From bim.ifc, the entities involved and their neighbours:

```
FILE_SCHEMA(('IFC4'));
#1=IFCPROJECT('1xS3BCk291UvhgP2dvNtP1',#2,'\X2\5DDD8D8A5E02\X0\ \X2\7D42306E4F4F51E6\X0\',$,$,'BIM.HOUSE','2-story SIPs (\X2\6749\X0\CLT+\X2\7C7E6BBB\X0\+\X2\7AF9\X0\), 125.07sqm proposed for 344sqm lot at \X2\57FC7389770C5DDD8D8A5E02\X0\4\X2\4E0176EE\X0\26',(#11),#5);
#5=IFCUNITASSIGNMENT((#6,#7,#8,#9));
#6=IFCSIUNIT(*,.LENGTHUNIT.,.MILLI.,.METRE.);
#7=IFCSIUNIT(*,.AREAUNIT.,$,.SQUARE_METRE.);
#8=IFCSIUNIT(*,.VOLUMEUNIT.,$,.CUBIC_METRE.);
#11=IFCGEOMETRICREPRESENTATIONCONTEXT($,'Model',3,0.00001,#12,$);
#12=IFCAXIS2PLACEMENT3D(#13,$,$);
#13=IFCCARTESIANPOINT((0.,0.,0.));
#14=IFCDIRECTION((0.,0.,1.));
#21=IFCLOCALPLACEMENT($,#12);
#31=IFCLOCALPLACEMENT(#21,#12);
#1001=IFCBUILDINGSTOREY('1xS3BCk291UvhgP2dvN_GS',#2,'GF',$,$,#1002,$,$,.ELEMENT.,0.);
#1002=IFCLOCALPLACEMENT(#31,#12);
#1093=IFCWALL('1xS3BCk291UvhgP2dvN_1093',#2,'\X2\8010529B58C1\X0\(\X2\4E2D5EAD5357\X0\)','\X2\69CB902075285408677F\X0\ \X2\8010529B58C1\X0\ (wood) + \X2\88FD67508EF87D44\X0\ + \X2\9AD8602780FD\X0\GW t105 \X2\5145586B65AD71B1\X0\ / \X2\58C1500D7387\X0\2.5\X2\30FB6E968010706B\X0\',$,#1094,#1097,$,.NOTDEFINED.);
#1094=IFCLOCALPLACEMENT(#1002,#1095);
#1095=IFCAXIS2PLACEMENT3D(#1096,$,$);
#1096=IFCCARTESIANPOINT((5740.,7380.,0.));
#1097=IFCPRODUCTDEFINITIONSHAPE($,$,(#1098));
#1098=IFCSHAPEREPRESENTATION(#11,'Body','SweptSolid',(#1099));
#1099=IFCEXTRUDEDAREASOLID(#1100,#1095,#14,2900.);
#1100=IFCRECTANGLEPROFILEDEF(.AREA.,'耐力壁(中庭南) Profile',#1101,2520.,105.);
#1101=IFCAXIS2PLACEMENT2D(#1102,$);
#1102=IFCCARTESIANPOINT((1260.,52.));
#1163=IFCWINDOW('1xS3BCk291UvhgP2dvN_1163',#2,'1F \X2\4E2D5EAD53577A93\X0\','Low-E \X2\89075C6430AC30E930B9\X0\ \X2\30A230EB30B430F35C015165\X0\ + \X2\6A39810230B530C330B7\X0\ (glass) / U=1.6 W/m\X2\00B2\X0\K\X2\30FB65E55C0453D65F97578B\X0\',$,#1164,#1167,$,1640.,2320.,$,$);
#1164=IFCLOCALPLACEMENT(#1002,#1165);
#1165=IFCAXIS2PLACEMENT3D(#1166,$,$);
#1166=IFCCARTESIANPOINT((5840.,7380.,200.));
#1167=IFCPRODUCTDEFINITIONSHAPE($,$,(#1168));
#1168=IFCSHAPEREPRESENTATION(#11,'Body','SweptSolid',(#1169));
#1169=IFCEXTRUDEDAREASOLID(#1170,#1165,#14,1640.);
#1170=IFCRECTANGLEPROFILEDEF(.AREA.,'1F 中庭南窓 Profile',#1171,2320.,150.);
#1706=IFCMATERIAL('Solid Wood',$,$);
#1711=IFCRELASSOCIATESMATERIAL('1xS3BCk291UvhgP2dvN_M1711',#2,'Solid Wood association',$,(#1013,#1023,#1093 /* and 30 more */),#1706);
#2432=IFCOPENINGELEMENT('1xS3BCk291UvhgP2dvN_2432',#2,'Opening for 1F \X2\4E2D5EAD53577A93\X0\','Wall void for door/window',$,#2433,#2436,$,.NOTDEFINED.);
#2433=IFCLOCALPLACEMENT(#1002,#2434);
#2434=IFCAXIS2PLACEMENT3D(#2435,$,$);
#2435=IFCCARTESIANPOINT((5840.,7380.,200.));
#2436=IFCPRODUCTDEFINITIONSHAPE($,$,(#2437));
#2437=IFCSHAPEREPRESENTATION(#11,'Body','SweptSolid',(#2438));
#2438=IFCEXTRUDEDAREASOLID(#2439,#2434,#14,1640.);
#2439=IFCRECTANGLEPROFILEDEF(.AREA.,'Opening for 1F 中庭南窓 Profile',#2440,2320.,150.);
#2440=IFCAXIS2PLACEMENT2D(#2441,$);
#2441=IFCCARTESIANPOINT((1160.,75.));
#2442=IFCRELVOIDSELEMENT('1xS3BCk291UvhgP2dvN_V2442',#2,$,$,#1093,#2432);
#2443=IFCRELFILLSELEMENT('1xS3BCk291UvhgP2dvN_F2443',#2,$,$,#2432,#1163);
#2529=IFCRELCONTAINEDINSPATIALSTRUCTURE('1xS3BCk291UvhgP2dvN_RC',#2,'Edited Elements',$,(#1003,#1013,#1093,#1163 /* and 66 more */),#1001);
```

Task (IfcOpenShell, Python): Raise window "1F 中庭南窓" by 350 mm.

```python
import numpy as np
import ifcopenshell
import ifcopenshell.api.geometry
import ifcopenshell.util.placement
import ifcopenshell.util.unit

model = ifcopenshell.open("bim.ifc")
unit_scale = ifcopenshell.util.unit.calculate_unit_scale(model)

window = model.by_guid("1xS3BCk291UvhgP2dvN_1163")
opening = window.FillsVoids[0].RelatingOpeningElement
dz = 0.35 / unit_scale

shift = np.array([0.0, 0.0, dz])
# The window is not placed relative to its opening, so move both.
for product in (opening, window):
    matrix = ifcopenshell.util.placement.get_local_placement(product.ObjectPlacement)
    matrix[:3, 3] += shift
    ifcopenshell.api.geometry.edit_object_placement(model, product=product, matrix=matrix, is_si=False)

print(f"moved by {dz * unit_scale:+.3f} m")

model.write("bim_edited.ifc")
```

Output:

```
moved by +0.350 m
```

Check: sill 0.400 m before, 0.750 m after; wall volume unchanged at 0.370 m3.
